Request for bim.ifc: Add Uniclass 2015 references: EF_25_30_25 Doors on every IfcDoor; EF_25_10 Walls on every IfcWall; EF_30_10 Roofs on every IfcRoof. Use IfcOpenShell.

First a look at what the model holds.

```python
import ifcopenshell

model = ifcopenshell.open("bim.ifc")
print(model.schema)
print("classifications:", [c.Name for c in model.by_type("IfcClassification")])
for ifc_class in ("IfcDoor", "IfcRoof", "IfcStair", "IfcWall", "IfcWindow"):
    print(ifc_class, len(model.by_type(ifc_class)))
```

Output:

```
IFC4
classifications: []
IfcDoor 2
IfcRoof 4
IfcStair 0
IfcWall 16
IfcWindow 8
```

```python
import ifcopenshell
import ifcopenshell.api.classification

model = ifcopenshell.open("bim.ifc")

system = ifcopenshell.api.classification.add_classification(model, classification="Uniclass 2015")

codes = {
    "IfcDoor": ("EF_25_30_25", "Doors"),
    "IfcWall": ("EF_25_10", "Walls"),
    "IfcRoof": ("EF_30_10", "Roofs"),
}
for ifc_class, (code, name) in codes.items():
    products = model.by_type(ifc_class)
    ifcopenshell.api.classification.add_reference(
        model, products=products, classification=system, identification=code, name=name
    )
    print(code, len(products))

model.write("bim_updated.ifc")
```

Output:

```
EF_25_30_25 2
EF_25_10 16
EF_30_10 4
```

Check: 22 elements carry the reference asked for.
